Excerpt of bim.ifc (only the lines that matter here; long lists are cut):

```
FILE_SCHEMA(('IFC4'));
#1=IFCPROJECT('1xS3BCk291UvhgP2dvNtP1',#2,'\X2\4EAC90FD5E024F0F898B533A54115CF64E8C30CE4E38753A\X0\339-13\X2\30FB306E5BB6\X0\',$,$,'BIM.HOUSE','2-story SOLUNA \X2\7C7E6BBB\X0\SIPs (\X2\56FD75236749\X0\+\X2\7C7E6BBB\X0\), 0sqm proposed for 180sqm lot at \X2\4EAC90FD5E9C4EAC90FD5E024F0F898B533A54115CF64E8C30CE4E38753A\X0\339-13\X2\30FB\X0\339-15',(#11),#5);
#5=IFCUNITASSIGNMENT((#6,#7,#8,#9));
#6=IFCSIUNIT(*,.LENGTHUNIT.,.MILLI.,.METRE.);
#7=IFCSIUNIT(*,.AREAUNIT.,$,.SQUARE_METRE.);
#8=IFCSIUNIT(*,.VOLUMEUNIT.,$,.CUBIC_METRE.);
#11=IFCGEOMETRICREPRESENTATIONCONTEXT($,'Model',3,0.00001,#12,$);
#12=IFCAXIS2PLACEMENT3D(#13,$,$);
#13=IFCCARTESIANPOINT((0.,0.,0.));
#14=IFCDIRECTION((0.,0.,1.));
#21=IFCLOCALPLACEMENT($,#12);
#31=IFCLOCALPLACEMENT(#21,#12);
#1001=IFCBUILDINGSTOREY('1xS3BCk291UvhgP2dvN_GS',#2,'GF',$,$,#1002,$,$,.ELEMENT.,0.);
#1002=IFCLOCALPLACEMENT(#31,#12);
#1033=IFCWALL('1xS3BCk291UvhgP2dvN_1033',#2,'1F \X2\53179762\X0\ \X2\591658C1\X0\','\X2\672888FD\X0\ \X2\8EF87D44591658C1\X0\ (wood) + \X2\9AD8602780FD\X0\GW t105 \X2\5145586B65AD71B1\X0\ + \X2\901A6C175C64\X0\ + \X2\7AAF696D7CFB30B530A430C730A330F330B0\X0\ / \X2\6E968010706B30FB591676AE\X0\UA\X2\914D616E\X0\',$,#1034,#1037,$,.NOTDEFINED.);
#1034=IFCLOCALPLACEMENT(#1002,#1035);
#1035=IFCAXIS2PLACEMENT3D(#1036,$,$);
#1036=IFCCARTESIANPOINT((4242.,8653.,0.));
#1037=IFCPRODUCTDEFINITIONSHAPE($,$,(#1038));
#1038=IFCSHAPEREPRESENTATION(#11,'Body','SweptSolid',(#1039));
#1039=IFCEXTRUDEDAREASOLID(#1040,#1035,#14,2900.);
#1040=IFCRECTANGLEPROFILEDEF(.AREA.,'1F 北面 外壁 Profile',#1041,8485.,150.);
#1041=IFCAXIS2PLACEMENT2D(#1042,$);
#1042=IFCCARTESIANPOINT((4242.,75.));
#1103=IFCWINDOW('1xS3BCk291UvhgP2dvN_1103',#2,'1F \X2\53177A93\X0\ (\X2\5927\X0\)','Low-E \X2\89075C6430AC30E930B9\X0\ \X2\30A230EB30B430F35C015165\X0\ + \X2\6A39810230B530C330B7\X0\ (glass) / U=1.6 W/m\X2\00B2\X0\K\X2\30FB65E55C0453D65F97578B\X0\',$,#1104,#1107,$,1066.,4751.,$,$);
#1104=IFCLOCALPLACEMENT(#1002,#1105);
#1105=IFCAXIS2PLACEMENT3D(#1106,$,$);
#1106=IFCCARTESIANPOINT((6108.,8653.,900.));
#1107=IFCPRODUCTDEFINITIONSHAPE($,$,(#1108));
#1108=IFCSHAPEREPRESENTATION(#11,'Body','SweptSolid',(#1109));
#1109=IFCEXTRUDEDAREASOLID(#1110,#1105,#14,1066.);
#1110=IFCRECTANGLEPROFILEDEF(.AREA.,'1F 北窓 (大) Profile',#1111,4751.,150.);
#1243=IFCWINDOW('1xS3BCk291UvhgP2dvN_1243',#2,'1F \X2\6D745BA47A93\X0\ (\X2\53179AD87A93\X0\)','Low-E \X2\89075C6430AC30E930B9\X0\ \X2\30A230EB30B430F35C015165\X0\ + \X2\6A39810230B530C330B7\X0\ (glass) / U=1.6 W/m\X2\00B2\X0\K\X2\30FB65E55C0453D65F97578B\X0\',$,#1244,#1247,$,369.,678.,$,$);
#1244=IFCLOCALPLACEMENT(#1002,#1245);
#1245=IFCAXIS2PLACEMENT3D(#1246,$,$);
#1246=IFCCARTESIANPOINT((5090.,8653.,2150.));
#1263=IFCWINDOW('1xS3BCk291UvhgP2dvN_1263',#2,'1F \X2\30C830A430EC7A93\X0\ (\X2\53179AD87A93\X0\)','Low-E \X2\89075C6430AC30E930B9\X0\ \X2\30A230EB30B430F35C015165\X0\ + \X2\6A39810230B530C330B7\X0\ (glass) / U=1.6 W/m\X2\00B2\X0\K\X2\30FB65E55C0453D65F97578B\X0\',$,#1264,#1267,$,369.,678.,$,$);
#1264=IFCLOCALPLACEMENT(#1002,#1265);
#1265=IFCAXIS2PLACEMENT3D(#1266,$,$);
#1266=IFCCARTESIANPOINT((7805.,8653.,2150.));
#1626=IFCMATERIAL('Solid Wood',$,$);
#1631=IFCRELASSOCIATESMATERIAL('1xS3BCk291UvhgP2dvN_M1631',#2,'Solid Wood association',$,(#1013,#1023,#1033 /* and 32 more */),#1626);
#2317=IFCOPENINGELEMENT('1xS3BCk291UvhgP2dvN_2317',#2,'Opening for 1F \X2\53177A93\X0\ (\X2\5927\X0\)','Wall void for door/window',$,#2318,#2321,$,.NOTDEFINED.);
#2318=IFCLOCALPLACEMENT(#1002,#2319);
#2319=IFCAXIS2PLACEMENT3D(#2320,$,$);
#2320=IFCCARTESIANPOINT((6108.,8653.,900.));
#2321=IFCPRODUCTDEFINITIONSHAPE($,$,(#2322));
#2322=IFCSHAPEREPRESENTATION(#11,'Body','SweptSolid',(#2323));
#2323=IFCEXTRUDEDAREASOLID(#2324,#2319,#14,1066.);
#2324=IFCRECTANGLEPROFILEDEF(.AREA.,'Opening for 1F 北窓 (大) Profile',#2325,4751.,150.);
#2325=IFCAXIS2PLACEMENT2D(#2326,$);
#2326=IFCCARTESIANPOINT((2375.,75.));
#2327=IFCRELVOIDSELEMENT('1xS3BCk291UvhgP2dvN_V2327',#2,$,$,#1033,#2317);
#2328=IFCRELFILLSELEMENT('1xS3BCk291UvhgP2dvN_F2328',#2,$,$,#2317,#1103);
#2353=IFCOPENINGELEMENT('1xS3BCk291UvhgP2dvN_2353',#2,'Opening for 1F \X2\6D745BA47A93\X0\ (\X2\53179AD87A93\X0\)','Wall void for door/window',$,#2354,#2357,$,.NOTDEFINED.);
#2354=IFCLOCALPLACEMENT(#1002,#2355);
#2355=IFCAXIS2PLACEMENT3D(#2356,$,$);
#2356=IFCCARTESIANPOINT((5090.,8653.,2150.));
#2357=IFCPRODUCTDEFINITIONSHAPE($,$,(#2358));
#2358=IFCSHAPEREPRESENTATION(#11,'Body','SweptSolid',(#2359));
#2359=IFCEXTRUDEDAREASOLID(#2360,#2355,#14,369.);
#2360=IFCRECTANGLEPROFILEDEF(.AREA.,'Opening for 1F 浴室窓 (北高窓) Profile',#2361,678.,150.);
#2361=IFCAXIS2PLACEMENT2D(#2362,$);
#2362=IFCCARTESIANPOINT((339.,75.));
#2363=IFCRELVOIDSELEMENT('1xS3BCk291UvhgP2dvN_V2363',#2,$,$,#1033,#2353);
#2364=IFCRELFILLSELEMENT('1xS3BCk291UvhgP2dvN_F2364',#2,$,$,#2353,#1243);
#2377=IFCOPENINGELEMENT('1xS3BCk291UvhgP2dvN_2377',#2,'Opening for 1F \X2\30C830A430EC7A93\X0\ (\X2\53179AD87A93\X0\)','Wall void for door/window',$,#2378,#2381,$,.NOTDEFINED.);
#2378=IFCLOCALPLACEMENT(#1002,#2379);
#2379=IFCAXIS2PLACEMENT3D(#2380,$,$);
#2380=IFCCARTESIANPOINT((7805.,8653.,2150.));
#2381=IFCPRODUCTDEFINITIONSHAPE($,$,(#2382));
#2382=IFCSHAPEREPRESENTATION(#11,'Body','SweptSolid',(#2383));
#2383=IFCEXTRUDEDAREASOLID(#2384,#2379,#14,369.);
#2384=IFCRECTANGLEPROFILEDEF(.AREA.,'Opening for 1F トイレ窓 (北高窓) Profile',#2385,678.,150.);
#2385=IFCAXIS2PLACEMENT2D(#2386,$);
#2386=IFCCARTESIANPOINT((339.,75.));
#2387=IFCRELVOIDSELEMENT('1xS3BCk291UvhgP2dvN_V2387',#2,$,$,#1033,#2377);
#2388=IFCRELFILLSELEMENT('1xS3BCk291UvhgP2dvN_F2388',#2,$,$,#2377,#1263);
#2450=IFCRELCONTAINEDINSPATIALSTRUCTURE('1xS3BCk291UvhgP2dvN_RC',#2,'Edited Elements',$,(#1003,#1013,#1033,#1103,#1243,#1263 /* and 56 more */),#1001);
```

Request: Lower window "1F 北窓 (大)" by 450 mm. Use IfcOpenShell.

```python
import numpy as np
import ifcopenshell
import ifcopenshell.api.geometry
import ifcopenshell.util.placement
import ifcopenshell.util.unit

model = ifcopenshell.open("bim.ifc")
unit_scale = ifcopenshell.util.unit.calculate_unit_scale(model)

window = model.by_guid("1xS3BCk291UvhgP2dvN_1103")
opening = window.FillsVoids[0].RelatingOpeningElement
dz = -0.45 / unit_scale

shift = np.array([0.0, 0.0, dz])
# The window is not placed relative to its opening, so move both.
for product in (opening, window):
    matrix = ifcopenshell.util.placement.get_local_placement(product.ObjectPlacement)
    matrix[:3, 3] += shift
    ifcopenshell.api.geometry.edit_object_placement(model, product=product, matrix=matrix, is_si=False)

print(f"moved by {dz * unit_scale:+.3f} m")

model.write("bim_updated.ifc")
```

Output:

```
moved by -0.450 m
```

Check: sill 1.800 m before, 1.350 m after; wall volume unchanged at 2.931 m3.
